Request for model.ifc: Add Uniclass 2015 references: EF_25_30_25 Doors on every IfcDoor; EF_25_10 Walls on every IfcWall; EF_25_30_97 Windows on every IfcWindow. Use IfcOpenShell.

First a look at what the model holds.

```python
import ifcopenshell

model = ifcopenshell.open("model.ifc")
print(model.schema)
print("classifications:", [c.Name for c in model.by_type("IfcClassification")])
for ifc_class in ("IfcDoor", "IfcRoof", "IfcStair", "IfcWall", "IfcWindow"):
    print(ifc_class, len(model.by_type(ifc_class)))
```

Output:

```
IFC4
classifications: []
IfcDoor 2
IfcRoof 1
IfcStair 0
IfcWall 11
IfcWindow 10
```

```python
import ifcopenshell
import ifcopenshell.api.classification

model = ifcopenshell.open("model.ifc")

system = ifcopenshell.api.classification.add_classification(model, classification="Uniclass 2015")

codes = {
    "IfcDoor": ("EF_25_30_25", "Doors"),
    "IfcWall": ("EF_25_10", "Walls"),
    "IfcWindow": ("EF_25_30_97", "Windows"),
}
for ifc_class, (code, name) in codes.items():
    products = model.by_type(ifc_class)
    ifcopenshell.api.classification.add_reference(
        model, products=products, classification=system, identification=code, name=name
    )
    print(code, len(products))

model.write("model-out.ifc")
```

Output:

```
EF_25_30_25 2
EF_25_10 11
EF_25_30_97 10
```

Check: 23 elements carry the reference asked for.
